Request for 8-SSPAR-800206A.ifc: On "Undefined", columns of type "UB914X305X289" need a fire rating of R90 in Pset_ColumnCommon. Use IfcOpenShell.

First a look at what the model holds.

```python
import ifcopenshell
import ifcopenshell.util.element

model = ifcopenshell.open("8-SSPAR-800206A.ifc")
print(model.schema)
storey = next(s for s in model.by_type("IfcBuildingStorey") if s.Name == "Undefined")
columns = [e for e in ifcopenshell.util.element.get_decomposition(storey) if e.is_a("IfcColumn")]
seen = {}
for e in columns:
    element_type = ifcopenshell.util.element.get_type(e)
    key = (element_type.Name if element_type != e and element_type else None, ifcopenshell.util.element.get_pset(e, "Pset_ColumnCommon", "FireRating"))
    seen[key] = seen.get(key, 0) + 1
for (name, value), count in sorted(seen.items(), key=str):
    print(count, "x", name, "|", value)
```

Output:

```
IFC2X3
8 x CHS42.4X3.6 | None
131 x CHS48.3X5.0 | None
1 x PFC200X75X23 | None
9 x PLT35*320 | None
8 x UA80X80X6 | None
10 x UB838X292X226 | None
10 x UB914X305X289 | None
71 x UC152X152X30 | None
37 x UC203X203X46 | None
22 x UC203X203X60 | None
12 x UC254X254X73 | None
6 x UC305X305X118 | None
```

```python
import ifcopenshell
import ifcopenshell.api.pset
import ifcopenshell.util.element

model = ifcopenshell.open("8-SSPAR-800206A.ifc")

storey = next(s for s in model.by_type("IfcBuildingStorey") if s.Name == "Undefined")
columns = [e for e in ifcopenshell.util.element.get_decomposition(storey) if e.is_a("IfcColumn")]

count = 0
for e in columns:
    element_type = ifcopenshell.util.element.get_type(e)
    if element_type in (None, e) or element_type.Name != "UB914X305X289":
        continue
    # add_pset returns the element's existing set when there is one.
    pset = ifcopenshell.api.pset.add_pset(model, product=e, name="Pset_ColumnCommon")
    ifcopenshell.api.pset.edit_pset(model, pset=pset, properties={"FireRating": "R90"})
    count += 1

print(count, "columns updated")

model.write("8-SSPAR-800206A_edited.ifc")
```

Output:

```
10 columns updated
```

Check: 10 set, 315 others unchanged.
